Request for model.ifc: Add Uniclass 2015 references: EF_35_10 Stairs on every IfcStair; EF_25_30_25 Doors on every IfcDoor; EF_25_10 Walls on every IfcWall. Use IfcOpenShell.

First a look at what the model holds.

```python
import ifcopenshell

model = ifcopenshell.open("model.ifc")
print(model.schema)
print("classifications:", [c.Name for c in model.by_type("IfcClassification")])
for ifc_class in ("IfcDoor", "IfcRoof", "IfcStair", "IfcWall", "IfcWindow"):
    print(ifc_class, len(model.by_type(ifc_class)))
```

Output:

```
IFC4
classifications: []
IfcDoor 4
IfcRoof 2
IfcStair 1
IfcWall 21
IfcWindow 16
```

```python
import ifcopenshell
import ifcopenshell.api.classification

model = ifcopenshell.open("model.ifc")

system = ifcopenshell.api.classification.add_classification(model, classification="Uniclass 2015")

codes = {
    "IfcStair": ("EF_35_10", "Stairs"),
    "IfcDoor": ("EF_25_30_25", "Doors"),
    "IfcWall": ("EF_25_10", "Walls"),
}
for ifc_class, (code, name) in codes.items():
    products = model.by_type(ifc_class)
    ifcopenshell.api.classification.add_reference(
        model, products=products, classification=system, identification=code, name=name
    )
    print(code, len(products))

model.write("model_v2.ifc")
```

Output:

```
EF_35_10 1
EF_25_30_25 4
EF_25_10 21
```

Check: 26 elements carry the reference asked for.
